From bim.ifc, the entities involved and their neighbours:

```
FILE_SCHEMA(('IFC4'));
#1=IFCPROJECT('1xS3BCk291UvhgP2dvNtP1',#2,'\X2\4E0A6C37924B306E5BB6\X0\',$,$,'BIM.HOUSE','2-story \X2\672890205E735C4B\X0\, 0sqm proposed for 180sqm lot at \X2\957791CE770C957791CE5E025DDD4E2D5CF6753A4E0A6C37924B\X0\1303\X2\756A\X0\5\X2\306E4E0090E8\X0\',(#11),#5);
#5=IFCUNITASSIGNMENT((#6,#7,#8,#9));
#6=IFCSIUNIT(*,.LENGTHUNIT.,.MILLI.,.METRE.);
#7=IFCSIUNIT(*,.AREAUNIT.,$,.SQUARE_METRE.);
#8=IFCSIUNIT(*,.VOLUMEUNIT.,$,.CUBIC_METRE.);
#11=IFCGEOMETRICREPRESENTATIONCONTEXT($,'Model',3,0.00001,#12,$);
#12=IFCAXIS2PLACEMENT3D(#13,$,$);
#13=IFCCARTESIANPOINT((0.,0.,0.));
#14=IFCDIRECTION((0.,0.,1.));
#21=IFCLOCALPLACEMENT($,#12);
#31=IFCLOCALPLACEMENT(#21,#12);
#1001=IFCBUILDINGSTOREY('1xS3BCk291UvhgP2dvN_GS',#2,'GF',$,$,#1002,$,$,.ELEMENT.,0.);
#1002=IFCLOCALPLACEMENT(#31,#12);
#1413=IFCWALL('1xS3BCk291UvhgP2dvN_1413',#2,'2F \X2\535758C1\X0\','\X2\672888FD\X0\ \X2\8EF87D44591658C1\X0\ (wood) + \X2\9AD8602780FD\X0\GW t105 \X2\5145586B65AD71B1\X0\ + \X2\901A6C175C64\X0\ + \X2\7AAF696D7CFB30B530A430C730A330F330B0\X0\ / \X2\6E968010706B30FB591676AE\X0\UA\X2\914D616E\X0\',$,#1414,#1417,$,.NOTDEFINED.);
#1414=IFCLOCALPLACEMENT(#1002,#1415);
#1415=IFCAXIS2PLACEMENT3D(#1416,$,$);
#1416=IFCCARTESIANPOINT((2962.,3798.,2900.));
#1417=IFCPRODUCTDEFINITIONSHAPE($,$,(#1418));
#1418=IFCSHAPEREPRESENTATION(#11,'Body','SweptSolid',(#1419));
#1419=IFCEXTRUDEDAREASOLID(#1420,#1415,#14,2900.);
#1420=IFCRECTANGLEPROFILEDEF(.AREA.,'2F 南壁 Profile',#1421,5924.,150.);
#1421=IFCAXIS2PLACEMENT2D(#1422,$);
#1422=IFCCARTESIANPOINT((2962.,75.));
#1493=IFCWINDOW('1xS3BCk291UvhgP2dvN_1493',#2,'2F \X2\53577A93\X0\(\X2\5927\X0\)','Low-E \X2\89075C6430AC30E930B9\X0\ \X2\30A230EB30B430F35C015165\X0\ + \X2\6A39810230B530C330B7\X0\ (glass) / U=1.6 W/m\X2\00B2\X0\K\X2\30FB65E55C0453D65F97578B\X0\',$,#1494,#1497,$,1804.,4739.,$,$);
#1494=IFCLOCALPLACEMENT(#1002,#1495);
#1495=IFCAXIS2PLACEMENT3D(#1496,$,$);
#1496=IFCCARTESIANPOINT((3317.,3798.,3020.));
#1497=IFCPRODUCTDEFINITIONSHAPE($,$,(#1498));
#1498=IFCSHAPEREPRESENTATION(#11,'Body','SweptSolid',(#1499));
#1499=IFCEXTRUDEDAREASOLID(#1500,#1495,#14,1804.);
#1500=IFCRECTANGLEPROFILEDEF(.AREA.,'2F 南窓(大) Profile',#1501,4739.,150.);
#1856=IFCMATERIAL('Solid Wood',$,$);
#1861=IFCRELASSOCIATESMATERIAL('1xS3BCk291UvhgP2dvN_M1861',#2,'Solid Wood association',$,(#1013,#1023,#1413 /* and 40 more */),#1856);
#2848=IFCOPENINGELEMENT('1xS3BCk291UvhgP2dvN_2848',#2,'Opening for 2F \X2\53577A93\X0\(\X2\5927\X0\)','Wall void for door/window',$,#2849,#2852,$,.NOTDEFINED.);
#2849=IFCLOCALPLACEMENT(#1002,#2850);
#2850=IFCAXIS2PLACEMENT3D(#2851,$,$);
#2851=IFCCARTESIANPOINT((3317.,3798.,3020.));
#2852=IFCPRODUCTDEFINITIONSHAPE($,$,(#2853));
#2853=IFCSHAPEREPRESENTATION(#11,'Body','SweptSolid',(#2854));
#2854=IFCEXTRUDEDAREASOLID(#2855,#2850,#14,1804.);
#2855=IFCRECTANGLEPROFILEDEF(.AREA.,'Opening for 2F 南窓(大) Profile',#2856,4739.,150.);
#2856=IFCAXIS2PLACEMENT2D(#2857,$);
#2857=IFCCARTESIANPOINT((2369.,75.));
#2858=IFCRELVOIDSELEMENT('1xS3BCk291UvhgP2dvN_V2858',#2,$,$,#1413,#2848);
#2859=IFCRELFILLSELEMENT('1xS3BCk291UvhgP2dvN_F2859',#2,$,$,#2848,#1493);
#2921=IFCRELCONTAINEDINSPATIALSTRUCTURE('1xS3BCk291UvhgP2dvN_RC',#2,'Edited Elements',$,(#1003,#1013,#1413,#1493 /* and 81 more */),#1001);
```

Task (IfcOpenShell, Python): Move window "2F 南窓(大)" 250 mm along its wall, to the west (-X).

```python
import ifcopenshell
import ifcopenshell.api.geometry
import ifcopenshell.util.placement
import ifcopenshell.util.unit

model = ifcopenshell.open("bim.ifc")
unit_scale = ifcopenshell.util.unit.calculate_unit_scale(model)

window = model.by_guid("1xS3BCk291UvhgP2dvN_1493")
opening = window.FillsVoids[0].RelatingOpeningElement
wall = opening.VoidsElements[0].RelatingBuildingElement

wall_matrix = ifcopenshell.util.placement.get_local_placement(wall.ObjectPlacement)
shift = wall_matrix[:3, 0] * -0.25 / unit_scale
before = ifcopenshell.util.placement.get_local_placement(window.ObjectPlacement)[:3, 3].copy()

# The window is not placed relative to its opening, so move both.
for product in (opening, window):
    matrix = ifcopenshell.util.placement.get_local_placement(product.ObjectPlacement)
    matrix[:3, 3] += shift
    ifcopenshell.api.geometry.edit_object_placement(model, product=product, matrix=matrix, is_si=False)

after = ifcopenshell.util.placement.get_local_placement(window.ObjectPlacement)[:3, 3]
print("window moved by", (after - before).round(3) + 0.0)

model.write("bim-out.ifc")
```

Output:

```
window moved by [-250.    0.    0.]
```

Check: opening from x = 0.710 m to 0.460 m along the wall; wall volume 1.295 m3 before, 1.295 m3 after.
